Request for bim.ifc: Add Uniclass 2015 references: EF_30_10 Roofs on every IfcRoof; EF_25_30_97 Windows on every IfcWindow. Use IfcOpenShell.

First a look at what the model holds.

```python
import ifcopenshell

model = ifcopenshell.open("bim.ifc")
print(model.schema)
print("classifications:", [c.Name for c in model.by_type("IfcClassification")])
for ifc_class in ("IfcDoor", "IfcRoof", "IfcStair", "IfcWall", "IfcWindow"):
    print(ifc_class, len(model.by_type(ifc_class)))
```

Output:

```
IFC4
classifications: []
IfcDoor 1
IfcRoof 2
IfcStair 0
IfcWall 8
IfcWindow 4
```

```python
import ifcopenshell
import ifcopenshell.api.classification

model = ifcopenshell.open("bim.ifc")

system = ifcopenshell.api.classification.add_classification(model, classification="Uniclass 2015")

codes = {
    "IfcRoof": ("EF_30_10", "Roofs"),
    "IfcWindow": ("EF_25_30_97", "Windows"),
}
for ifc_class, (code, name) in codes.items():
    products = model.by_type(ifc_class)
    ifcopenshell.api.classification.add_reference(
        model, products=products, classification=system, identification=code, name=name
    )
    print(code, len(products))

model.write("bim-out.ifc")
```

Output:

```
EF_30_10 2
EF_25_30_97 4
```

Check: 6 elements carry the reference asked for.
